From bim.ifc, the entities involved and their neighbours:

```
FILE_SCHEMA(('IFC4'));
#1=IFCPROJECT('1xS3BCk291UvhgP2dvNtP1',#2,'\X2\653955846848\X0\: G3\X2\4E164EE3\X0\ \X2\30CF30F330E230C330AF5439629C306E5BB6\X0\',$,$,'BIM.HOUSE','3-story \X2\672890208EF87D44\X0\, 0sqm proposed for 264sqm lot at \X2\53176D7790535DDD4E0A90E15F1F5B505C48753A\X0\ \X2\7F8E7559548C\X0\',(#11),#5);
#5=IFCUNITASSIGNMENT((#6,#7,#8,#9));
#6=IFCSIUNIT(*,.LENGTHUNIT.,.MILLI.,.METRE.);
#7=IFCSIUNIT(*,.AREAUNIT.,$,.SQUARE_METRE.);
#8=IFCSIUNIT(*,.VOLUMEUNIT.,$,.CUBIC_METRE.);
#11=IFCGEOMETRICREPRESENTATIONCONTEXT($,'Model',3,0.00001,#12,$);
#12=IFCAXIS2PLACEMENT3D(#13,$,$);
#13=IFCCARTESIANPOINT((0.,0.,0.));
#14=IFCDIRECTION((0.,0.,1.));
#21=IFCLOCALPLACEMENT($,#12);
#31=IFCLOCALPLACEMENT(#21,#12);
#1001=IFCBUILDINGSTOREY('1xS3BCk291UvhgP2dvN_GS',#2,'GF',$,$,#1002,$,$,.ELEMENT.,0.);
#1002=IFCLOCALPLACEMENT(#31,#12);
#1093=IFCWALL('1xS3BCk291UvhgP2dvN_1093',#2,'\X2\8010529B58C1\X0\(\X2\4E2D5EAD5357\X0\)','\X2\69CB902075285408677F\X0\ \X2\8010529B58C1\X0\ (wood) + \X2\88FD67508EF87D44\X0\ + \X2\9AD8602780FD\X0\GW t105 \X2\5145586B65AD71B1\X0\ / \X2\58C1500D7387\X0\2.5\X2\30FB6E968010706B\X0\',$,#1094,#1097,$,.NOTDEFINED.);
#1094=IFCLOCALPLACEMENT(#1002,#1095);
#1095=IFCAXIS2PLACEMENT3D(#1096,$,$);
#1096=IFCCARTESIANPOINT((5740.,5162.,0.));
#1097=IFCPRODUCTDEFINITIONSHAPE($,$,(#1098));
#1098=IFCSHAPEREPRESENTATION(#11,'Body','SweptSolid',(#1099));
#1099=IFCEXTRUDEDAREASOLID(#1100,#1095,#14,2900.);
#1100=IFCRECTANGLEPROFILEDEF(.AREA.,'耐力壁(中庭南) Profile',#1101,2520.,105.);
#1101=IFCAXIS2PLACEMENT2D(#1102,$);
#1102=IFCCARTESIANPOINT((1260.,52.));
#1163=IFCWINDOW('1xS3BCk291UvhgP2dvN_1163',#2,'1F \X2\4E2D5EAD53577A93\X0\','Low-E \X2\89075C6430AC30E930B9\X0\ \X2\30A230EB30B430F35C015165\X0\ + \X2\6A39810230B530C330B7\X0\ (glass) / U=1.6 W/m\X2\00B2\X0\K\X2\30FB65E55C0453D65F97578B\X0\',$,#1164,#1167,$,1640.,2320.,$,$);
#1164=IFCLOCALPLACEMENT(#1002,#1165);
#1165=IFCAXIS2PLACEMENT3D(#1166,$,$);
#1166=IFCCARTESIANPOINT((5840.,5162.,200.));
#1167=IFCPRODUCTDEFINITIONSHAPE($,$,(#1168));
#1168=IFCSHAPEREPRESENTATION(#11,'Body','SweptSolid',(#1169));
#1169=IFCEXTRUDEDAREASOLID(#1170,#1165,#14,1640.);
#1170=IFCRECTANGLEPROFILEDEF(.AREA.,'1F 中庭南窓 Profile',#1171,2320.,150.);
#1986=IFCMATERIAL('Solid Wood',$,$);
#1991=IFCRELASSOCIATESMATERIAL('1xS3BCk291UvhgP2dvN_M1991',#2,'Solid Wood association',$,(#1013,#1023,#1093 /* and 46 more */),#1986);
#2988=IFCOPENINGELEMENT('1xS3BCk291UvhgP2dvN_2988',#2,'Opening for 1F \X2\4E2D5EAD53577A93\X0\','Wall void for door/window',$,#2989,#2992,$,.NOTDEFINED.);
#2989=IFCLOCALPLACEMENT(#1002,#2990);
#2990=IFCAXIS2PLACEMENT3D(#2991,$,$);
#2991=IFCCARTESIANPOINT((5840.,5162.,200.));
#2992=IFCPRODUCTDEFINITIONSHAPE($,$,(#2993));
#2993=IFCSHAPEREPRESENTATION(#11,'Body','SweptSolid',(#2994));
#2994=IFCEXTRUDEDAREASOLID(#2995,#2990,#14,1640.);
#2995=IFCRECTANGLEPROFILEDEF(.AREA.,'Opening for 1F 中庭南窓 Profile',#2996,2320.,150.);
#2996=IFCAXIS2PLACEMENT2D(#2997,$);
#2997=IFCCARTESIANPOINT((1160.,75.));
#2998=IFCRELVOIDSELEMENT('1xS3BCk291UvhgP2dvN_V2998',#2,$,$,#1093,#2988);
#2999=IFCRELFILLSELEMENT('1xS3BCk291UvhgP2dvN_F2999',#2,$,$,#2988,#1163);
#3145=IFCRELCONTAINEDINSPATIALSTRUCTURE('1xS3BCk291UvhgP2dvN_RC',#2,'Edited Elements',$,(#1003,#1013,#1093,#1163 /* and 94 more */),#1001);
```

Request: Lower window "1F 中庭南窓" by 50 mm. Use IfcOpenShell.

```python
import numpy as np
import ifcopenshell
import ifcopenshell.api.geometry
import ifcopenshell.util.placement
import ifcopenshell.util.unit

model = ifcopenshell.open("bim.ifc")
unit_scale = ifcopenshell.util.unit.calculate_unit_scale(model)

window = model.by_id(1163)
opening = window.FillsVoids[0].RelatingOpeningElement
dz = -0.05 / unit_scale

shift = np.array([0.0, 0.0, dz])
# The window is not placed relative to its opening, so move both.
for product in (opening, window):
    matrix = ifcopenshell.util.placement.get_local_placement(product.ObjectPlacement)
    matrix[:3, 3] += shift
    ifcopenshell.api.geometry.edit_object_placement(model, product=product, matrix=matrix, is_si=False)

print(f"moved by {dz * unit_scale:+.3f} m")

model.write("bim-out.ifc")
```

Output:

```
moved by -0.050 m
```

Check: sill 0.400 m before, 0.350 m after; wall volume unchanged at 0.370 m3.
